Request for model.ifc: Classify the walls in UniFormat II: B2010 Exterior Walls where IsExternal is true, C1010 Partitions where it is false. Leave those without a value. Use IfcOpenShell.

First a look at what the model holds.

```python
import ifcopenshell
import ifcopenshell.util.element

model = ifcopenshell.open("model.ifc")
print(model.schema)
print("classifications:", [c.Name for c in model.by_type("IfcClassification")])
values = [ifcopenshell.util.element.get_pset(e, "Pset_WallCommon", "IsExternal") for e in model.by_type("IfcWall")]
for value in (True, False, None):
    print("IsExternal", value, values.count(value))
```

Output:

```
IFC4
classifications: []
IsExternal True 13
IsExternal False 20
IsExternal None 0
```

```python
import ifcopenshell
import ifcopenshell.api.classification
import ifcopenshell.util.element

model = ifcopenshell.open("model.ifc")

system = ifcopenshell.api.classification.add_classification(model, classification="UniFormat II")

walls = model.by_type("IfcWall")
external = {e: ifcopenshell.util.element.get_pset(e, "Pset_WallCommon", "IsExternal") for e in walls}
for flag, code, name in ((True, "B2010", "Exterior Walls"), (False, "C1010", "Partitions")):
    products = [e for e in walls if external[e] is flag]
    ifcopenshell.api.classification.add_reference(
        model, products=products, classification=system, identification=code, name=name
    )
    print(code, len(products))

model.write("model-out.ifc")
```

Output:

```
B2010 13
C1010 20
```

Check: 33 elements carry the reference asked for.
